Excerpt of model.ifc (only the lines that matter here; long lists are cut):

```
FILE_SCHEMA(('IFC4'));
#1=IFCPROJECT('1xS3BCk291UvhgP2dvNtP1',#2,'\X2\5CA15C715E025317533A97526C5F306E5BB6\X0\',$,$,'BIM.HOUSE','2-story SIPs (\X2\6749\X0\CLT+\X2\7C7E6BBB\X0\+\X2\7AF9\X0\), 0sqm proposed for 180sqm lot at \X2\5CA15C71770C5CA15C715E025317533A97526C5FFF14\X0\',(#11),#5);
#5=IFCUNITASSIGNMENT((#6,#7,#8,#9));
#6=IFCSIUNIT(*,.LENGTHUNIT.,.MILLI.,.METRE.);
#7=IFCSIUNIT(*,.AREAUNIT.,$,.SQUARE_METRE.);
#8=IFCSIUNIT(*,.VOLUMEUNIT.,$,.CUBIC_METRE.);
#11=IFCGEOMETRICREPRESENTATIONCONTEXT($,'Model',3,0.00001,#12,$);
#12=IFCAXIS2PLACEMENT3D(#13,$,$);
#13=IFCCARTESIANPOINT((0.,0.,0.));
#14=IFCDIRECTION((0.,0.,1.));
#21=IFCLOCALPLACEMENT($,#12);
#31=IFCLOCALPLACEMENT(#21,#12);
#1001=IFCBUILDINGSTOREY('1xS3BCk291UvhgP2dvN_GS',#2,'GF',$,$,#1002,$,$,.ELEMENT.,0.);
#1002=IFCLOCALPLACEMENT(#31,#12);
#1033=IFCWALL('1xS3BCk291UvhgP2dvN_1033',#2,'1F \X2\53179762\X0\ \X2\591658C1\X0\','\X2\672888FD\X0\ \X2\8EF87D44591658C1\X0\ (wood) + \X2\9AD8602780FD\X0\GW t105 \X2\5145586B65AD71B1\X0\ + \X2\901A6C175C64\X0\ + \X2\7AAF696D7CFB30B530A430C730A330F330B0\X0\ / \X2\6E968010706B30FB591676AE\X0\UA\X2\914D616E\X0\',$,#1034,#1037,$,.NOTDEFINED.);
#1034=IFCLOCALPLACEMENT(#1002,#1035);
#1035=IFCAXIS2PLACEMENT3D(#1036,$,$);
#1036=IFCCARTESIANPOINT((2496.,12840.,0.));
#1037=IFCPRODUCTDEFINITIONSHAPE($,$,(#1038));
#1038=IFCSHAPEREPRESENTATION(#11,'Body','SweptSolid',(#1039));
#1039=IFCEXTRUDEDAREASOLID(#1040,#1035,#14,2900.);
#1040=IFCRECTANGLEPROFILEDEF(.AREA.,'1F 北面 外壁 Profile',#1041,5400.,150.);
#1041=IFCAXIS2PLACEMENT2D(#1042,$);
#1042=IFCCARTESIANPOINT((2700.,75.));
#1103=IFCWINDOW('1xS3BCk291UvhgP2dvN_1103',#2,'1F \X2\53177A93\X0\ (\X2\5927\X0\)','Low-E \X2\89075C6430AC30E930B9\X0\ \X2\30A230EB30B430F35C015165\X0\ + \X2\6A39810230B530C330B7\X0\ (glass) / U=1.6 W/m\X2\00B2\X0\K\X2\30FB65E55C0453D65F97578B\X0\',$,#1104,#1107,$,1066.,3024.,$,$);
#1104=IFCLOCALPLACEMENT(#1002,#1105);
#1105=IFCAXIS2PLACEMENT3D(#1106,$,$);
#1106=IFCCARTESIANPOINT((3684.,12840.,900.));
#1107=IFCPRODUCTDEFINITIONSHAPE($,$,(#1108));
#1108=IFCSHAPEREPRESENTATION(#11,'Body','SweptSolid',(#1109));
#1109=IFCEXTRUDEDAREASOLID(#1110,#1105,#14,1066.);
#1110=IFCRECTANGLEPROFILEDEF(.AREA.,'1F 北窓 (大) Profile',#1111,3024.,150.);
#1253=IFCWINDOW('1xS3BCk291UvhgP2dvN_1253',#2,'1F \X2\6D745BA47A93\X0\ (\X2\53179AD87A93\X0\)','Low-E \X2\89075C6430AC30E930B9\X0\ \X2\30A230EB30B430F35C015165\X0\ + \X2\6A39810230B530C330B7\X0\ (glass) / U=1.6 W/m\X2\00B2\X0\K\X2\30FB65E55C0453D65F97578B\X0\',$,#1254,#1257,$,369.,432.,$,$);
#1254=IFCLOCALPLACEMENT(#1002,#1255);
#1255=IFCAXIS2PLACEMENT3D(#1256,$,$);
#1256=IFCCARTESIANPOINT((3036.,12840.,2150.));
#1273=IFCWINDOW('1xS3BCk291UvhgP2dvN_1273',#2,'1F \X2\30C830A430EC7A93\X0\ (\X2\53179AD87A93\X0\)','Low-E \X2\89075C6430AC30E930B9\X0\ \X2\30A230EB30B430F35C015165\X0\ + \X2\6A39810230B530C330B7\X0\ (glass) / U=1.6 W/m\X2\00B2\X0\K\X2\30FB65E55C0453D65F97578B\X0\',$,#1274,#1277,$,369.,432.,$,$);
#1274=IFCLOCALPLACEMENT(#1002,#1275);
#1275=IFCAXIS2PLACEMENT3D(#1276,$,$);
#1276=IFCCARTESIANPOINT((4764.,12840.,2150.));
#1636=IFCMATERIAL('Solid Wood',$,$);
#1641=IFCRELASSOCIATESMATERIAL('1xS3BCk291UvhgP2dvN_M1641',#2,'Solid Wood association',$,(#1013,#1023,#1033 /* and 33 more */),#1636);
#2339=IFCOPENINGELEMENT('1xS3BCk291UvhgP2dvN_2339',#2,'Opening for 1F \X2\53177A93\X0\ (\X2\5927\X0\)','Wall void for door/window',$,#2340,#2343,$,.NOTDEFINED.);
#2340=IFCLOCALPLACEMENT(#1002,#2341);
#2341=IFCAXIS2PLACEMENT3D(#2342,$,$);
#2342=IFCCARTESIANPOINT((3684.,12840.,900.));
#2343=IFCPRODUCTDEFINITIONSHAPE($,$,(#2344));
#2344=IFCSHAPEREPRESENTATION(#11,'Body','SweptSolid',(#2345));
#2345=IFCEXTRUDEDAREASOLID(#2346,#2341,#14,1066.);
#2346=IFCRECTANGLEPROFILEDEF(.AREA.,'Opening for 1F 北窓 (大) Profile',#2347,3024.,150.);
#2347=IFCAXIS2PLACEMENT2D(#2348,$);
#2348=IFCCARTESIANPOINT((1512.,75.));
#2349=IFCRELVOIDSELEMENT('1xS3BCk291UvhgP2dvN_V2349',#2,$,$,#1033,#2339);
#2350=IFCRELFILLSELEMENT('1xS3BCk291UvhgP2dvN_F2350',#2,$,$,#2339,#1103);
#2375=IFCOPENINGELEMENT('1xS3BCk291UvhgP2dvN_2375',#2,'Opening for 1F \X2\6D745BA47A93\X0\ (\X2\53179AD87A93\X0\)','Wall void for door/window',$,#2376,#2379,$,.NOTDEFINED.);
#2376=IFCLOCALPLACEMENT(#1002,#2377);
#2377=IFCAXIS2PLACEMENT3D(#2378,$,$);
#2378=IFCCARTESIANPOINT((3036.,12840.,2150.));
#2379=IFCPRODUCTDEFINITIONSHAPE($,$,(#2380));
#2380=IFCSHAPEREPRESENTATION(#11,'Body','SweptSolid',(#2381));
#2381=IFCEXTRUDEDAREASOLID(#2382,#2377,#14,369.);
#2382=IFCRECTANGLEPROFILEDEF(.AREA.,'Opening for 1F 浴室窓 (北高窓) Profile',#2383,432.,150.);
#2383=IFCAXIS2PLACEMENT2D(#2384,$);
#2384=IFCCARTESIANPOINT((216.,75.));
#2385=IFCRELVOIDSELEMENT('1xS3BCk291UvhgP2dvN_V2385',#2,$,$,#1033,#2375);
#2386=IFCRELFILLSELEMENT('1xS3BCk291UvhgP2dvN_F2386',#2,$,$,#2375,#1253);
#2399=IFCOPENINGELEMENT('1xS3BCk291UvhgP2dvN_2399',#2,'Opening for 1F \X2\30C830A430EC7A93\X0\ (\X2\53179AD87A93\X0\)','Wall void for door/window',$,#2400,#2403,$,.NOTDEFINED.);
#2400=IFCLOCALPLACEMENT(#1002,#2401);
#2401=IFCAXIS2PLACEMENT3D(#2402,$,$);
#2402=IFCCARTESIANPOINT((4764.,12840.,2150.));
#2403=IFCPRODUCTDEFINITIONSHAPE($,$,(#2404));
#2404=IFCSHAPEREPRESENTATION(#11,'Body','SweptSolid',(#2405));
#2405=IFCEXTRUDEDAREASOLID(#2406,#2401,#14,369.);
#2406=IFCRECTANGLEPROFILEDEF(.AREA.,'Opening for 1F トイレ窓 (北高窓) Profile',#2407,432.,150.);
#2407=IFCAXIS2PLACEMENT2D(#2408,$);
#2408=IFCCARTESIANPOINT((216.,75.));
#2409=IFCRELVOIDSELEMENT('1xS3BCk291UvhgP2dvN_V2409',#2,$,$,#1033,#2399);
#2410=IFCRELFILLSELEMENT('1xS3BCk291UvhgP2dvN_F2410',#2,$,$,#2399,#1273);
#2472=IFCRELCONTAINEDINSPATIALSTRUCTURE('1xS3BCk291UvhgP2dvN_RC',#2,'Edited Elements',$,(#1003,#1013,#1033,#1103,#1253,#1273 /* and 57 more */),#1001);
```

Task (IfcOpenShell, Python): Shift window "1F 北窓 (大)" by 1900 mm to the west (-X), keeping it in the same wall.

```python
import ifcopenshell
import ifcopenshell.api.geometry
import ifcopenshell.util.placement
import ifcopenshell.util.unit

model = ifcopenshell.open("model.ifc")
unit_scale = ifcopenshell.util.unit.calculate_unit_scale(model)

window = model.by_id(1103)
opening = window.FillsVoids[0].RelatingOpeningElement
wall = opening.VoidsElements[0].RelatingBuildingElement

wall_matrix = ifcopenshell.util.placement.get_local_placement(wall.ObjectPlacement)
shift = wall_matrix[:3, 0] * -1.9 / unit_scale
before = ifcopenshell.util.placement.get_local_placement(window.ObjectPlacement)[:3, 3].copy()

# The window is not placed relative to its opening, so move both.
for product in (opening, window):
    matrix = ifcopenshell.util.placement.get_local_placement(product.ObjectPlacement)
    matrix[:3, 3] += shift
    ifcopenshell.api.geometry.edit_object_placement(model, product=product, matrix=matrix, is_si=False)

after = ifcopenshell.util.placement.get_local_placement(window.ObjectPlacement)[:3, 3]
print("window moved by", (after - before).round(3) + 0.0)

model.write("model_edited.ifc")
```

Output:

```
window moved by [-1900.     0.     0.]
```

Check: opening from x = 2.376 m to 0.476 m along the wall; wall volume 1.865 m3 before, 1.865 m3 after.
